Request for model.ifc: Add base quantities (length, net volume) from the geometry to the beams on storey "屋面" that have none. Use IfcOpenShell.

First a look at what the model holds.

```python
import ifcopenshell
import ifcopenshell.util.element
import ifcopenshell.util.unit

model = ifcopenshell.open("model.ifc")
print(model.schema)
for unit_type in ("LENGTHUNIT", "AREAUNIT", "VOLUMEUNIT"):
    print(unit_type, ifcopenshell.util.unit.calculate_unit_scale(model, unit_type))
storey = next(s for s in model.by_type("IfcBuildingStorey") if s.Name == "屋面")
beams = [e for e in ifcopenshell.util.element.get_decomposition(storey) if e.is_a("IfcBeam")]
for e in sorted(beams, key=lambda e: e.id()):
    print(e.id(), e.is_a(), e.Name, list(ifcopenshell.util.element.get_psets(e, qtos_only=True)), sep=" | ")
```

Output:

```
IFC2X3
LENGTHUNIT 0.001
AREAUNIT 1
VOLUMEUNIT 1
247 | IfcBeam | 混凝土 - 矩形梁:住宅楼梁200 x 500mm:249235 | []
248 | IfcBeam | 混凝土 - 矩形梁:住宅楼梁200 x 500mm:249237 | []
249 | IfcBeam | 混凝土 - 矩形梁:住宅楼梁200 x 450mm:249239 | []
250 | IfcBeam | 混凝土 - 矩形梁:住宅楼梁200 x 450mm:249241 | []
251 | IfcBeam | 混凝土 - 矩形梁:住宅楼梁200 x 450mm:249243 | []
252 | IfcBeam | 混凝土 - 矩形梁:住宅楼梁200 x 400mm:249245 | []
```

```python
import ifcopenshell
import ifcopenshell.api.pset
import ifcopenshell.geom
import ifcopenshell.util.element
import ifcopenshell.util.shape
import ifcopenshell.util.unit

model = ifcopenshell.open("model.ifc")
unit_scale = ifcopenshell.util.unit.calculate_unit_scale(model)
volume_scale = ifcopenshell.util.unit.calculate_unit_scale(model, "VOLUMEUNIT")
settings = ifcopenshell.geom.settings()

storey = next(s for s in model.by_type("IfcBuildingStorey") if s.Name == "屋面")
beams = [e for e in ifcopenshell.util.element.get_decomposition(storey) if e.is_a("IfcBeam")]

for e in sorted(beams, key=lambda e: e.id()):
    if ifcopenshell.util.element.get_psets(e, qtos_only=True, should_inherit=False):
        continue
    # Geometry comes back in metres, in the element's own axes.
    shape = ifcopenshell.geom.create_shape(settings, e)
    values = {
        "Length": ifcopenshell.util.shape.get_max_xyz(shape.geometry) / unit_scale,
        "NetVolume": ifcopenshell.util.shape.get_volume(shape.geometry) / volume_scale,
    }
    qto = ifcopenshell.api.pset.add_qto(model, product=e, name="BaseQuantities")
    ifcopenshell.api.pset.edit_qto(model, qto=qto, properties=values)
    print(e.id(), {k: round(v, 3) for k, v in values.items()})

model.write("model_updated.ifc")
```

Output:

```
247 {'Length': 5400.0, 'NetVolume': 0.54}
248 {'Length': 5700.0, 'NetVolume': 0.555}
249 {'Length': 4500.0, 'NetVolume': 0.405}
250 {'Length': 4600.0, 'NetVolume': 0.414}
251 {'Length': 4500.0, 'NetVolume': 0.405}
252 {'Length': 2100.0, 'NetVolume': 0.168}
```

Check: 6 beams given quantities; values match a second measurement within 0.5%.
